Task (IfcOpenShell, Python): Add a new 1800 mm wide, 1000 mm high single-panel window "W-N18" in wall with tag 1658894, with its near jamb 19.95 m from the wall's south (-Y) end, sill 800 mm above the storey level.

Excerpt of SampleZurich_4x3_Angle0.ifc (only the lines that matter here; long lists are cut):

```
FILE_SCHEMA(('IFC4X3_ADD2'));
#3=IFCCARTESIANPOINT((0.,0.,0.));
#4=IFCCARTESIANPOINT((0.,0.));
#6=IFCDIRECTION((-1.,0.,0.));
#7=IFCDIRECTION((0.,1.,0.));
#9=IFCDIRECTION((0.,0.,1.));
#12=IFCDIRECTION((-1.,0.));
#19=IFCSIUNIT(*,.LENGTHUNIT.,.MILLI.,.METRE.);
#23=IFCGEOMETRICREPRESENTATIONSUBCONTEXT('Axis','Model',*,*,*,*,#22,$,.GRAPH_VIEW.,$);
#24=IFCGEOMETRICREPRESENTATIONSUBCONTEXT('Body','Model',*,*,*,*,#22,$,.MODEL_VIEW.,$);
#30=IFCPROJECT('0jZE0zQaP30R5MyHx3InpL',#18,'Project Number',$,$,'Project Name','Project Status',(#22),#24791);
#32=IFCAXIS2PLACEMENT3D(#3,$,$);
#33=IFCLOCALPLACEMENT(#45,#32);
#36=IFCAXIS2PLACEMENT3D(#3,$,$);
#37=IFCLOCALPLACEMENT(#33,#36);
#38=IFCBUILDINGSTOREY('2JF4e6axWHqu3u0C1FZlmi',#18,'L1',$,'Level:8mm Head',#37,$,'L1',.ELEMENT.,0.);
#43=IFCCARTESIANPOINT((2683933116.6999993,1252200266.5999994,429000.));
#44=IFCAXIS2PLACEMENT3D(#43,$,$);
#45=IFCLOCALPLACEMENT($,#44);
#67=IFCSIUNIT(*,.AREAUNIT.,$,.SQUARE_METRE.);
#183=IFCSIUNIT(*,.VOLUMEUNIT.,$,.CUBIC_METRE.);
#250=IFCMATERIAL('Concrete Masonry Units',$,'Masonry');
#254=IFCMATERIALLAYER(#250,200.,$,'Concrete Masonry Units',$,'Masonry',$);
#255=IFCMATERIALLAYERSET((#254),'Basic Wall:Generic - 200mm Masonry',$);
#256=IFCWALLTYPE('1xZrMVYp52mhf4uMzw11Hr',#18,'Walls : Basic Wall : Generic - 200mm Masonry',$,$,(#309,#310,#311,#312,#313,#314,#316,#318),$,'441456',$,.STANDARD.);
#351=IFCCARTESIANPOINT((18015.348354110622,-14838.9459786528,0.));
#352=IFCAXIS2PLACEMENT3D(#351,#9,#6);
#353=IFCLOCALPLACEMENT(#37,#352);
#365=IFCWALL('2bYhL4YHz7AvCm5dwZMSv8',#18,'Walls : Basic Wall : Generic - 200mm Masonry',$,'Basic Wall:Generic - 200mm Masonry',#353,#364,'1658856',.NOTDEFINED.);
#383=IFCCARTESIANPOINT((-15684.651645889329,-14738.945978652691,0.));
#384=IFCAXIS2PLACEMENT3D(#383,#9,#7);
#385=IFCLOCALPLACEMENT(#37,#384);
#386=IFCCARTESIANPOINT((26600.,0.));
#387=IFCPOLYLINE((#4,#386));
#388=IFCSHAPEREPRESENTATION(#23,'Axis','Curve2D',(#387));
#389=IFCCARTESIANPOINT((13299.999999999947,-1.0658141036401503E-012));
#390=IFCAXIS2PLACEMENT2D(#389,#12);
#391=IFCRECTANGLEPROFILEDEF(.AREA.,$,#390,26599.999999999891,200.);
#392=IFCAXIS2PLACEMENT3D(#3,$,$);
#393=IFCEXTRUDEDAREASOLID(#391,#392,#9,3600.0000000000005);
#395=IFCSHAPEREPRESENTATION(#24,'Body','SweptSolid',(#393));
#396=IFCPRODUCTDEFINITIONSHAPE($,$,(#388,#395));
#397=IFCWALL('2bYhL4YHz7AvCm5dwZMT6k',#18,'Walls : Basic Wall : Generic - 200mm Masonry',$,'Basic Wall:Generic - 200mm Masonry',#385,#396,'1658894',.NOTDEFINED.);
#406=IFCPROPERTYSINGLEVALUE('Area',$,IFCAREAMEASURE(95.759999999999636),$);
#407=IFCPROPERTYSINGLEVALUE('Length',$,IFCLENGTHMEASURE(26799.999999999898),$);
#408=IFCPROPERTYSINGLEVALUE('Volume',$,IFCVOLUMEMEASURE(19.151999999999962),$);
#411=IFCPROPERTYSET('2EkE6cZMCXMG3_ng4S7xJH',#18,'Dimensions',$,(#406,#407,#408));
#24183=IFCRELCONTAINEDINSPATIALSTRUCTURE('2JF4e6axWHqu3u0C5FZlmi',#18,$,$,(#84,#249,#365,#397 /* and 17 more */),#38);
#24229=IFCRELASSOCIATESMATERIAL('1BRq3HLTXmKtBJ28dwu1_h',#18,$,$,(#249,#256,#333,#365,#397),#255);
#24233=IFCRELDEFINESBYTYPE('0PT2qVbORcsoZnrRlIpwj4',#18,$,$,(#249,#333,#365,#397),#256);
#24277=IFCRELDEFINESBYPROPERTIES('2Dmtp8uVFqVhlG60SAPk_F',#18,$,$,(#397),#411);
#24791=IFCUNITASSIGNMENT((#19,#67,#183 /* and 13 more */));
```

```python
import numpy as np
import ifcopenshell
import ifcopenshell.api.feature
import ifcopenshell.api.geometry
import ifcopenshell.api.pset
import ifcopenshell.api.root
import ifcopenshell.api.spatial
import ifcopenshell.geom
import ifcopenshell.util.element
import ifcopenshell.util.placement
import ifcopenshell.util.representation
import ifcopenshell.util.shape
import ifcopenshell.util.unit

model = ifcopenshell.open("SampleZurich_4x3_Angle0.ifc")
unit_scale = ifcopenshell.util.unit.calculate_unit_scale(model)
area_scale = ifcopenshell.util.unit.calculate_unit_scale(model, "AREAUNIT")
volume_scale = ifcopenshell.util.unit.calculate_unit_scale(model, "VOLUMEUNIT")
settings = ifcopenshell.geom.settings()


def volume(element):
    """Net volume in cubic metres, openings subtracted."""
    shape = ifcopenshell.geom.create_shape(settings, element)
    return ifcopenshell.util.shape.get_volume(shape.geometry)


wall = model.by_id(397)
storey = ifcopenshell.util.element.get_container(wall, ifc_class="IfcBuildingStorey")
context = ifcopenshell.util.representation.get_context(model, "Model", "Body", "MODEL_VIEW")
before = volume(wall)

width, height, from_end, sill = 1.8, 1, 19.95, 0.8  # metres

# The wall runs along its own X axis, and the end named is its -X end.
wall_shape = ifcopenshell.geom.create_shape(settings, wall)
x, y, z = ifcopenshell.util.shape.get_vertices(wall_shape.geometry).T
start = x.min() + from_end
face, thickness = float(y.min()), float(y.max() - y.min())
wall_matrix = ifcopenshell.util.placement.get_local_placement(wall.ObjectPlacement)
level = ifcopenshell.util.placement.get_local_placement(storey.ObjectPlacement)[2, 3]


def in_wall(x, y):
    """Placement at x, y metres in the wall's axes, at sill height."""
    matrix = wall_matrix.copy()
    matrix[:, 3] = wall_matrix @ np.array([x / unit_scale, y / unit_scale, 0.0, 1.0])
    matrix[2, 3] = level + sill / unit_scale
    return matrix


# Opening: a box that overshoots both wall faces by 50 mm.
opening = ifcopenshell.api.root.create_entity(model, ifc_class="IfcOpeningElement", predefined_type="OPENING")
box = ifcopenshell.api.geometry.add_wall_representation(
    model, context=context, length=width, height=height, thickness=thickness + 0.1
)
ifcopenshell.api.geometry.assign_representation(model, product=opening, representation=box)
ifcopenshell.api.geometry.edit_object_placement(model, product=opening, matrix=in_wall(start, face - 0.05), is_si=False)
ifcopenshell.api.feature.add_feature(model, feature=opening, element=wall)

window = ifcopenshell.api.root.create_entity(model, ifc_class="IfcWindow", name="W-N18", predefined_type="WINDOW")
window.OverallWidth, window.OverallHeight = width / unit_scale, height / unit_scale
window.PartitioningType = "SINGLE_PANEL"
body = ifcopenshell.api.geometry.add_window_representation(
    model,
    context=context,
    overall_width=window.OverallWidth,
    overall_height=window.OverallHeight,
    partition_type="SINGLE_PANEL",
)
ifcopenshell.api.geometry.assign_representation(model, product=window, representation=body)
ifcopenshell.api.spatial.assign_container(model, products=[window], relating_structure=storey)
ifcopenshell.api.feature.add_filling(model, opening=opening, element=window)

# Centre the window in the wall's thickness.
ifcopenshell.api.geometry.edit_object_placement(model, product=window, matrix=in_wall(start, face), is_si=False)
window_shape = ifcopenshell.geom.create_shape(settings, window)
depth = ifcopenshell.util.shape.get_vertices(window_shape.geometry)[:, 1]
offset = face + thickness / 2 - (depth.min() + depth.max()) / 2
ifcopenshell.api.geometry.edit_object_placement(model, product=window, matrix=in_wall(start, offset), is_si=False)

after = volume(wall)

# Update the wall's stored quantities.
pset = model.by_id(ifcopenshell.util.element.get_pset(wall, "Dimensions", should_inherit=False)["id"])
ifcopenshell.api.pset.edit_pset(model, pset=pset, properties={
    "Area": model.create_entity("IfcAreaMeasure", after / thickness / area_scale),
    "Volume": model.create_entity("IfcVolumeMeasure", after / volume_scale),
})

print(f"wall volume {before:.3f} -> {after:.3f} m3")

model.write("SampleZurich_4x3_Angle0_edited.ifc")
```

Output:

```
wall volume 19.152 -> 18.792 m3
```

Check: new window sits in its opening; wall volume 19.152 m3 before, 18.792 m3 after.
